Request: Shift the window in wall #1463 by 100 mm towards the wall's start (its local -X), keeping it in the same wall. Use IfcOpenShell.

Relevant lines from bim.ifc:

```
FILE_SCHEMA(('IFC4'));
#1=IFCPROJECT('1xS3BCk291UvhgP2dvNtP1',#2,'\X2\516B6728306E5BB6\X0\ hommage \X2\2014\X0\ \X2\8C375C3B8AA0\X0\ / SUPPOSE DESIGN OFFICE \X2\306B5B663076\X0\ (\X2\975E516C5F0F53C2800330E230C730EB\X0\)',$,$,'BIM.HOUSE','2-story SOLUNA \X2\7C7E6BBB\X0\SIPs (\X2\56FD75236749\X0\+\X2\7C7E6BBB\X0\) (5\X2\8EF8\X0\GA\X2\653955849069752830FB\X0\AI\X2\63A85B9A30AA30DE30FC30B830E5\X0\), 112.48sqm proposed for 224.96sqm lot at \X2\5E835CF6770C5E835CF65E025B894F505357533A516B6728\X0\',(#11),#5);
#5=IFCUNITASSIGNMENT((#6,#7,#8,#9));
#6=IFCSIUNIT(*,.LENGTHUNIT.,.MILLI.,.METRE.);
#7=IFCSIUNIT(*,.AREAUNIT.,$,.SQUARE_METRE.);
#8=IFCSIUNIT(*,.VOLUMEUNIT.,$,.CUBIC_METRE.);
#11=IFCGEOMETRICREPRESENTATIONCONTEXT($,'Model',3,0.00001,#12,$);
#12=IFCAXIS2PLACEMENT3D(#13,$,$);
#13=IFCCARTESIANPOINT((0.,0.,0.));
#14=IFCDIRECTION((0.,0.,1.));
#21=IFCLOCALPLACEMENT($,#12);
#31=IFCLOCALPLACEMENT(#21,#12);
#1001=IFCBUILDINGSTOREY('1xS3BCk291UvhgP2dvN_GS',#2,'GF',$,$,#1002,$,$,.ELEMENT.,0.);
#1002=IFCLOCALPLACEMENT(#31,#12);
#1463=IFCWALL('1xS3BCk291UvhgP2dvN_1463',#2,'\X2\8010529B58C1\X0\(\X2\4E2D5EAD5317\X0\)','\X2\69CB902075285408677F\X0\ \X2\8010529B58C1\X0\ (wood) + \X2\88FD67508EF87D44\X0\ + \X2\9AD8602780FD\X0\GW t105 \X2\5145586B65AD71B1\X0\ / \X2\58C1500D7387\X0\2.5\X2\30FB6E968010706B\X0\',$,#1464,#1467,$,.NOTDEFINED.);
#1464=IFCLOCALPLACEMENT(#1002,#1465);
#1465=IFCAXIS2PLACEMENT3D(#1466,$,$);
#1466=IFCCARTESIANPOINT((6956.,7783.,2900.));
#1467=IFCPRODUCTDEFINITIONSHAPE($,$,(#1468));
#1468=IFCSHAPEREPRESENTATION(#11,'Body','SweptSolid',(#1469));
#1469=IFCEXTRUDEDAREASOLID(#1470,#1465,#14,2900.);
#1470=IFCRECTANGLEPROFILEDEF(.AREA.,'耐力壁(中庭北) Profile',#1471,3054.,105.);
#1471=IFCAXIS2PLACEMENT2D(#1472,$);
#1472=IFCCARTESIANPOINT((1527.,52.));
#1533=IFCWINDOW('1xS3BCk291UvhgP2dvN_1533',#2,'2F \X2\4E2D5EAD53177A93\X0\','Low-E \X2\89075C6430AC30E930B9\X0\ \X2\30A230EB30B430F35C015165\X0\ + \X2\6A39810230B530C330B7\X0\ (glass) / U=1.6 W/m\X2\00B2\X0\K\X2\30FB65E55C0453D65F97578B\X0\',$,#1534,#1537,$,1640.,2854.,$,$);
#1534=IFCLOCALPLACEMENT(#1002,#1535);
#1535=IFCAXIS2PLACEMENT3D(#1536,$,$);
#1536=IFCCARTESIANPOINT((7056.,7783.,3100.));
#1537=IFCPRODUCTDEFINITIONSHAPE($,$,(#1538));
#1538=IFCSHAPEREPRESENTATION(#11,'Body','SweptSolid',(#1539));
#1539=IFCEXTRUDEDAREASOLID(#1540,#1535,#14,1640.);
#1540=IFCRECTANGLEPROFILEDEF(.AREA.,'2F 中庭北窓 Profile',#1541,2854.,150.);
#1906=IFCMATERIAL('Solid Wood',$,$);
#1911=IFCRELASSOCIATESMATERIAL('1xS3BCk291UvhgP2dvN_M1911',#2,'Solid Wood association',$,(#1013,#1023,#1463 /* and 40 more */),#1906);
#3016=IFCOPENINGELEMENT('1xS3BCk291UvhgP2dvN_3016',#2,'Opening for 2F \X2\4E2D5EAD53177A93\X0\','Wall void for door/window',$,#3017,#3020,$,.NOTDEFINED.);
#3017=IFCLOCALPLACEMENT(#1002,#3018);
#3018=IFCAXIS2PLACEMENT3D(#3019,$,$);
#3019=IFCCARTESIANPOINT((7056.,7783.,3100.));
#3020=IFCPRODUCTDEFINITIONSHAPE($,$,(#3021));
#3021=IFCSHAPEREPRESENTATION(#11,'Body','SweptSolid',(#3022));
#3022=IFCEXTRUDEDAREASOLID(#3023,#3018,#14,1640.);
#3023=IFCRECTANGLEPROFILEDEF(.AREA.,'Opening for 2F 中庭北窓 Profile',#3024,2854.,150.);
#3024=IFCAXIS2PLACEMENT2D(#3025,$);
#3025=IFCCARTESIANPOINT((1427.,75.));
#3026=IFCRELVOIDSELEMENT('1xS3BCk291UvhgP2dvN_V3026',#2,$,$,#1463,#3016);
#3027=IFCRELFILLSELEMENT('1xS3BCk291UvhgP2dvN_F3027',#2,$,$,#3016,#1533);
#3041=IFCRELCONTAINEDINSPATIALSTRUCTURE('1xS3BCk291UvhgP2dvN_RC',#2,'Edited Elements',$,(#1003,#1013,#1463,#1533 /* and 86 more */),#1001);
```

```python
import ifcopenshell
import ifcopenshell.api.geometry
import ifcopenshell.util.placement
import ifcopenshell.util.unit

model = ifcopenshell.open("bim.ifc")
unit_scale = ifcopenshell.util.unit.calculate_unit_scale(model)

window = model.by_guid("1xS3BCk291UvhgP2dvN_1533")
opening = window.FillsVoids[0].RelatingOpeningElement
wall = opening.VoidsElements[0].RelatingBuildingElement

wall_matrix = ifcopenshell.util.placement.get_local_placement(wall.ObjectPlacement)
shift = wall_matrix[:3, 0] * -0.1 / unit_scale
before = ifcopenshell.util.placement.get_local_placement(window.ObjectPlacement)[:3, 3].copy()

# The window is not placed relative to its opening, so move both.
for product in (opening, window):
    matrix = ifcopenshell.util.placement.get_local_placement(product.ObjectPlacement)
    matrix[:3, 3] += shift
    ifcopenshell.api.geometry.edit_object_placement(model, product=product, matrix=matrix, is_si=False)

after = ifcopenshell.util.placement.get_local_placement(window.ObjectPlacement)[:3, 3]
print("window moved by", (after - before).round(3) + 0.0)

model.write("bim-out.ifc")
```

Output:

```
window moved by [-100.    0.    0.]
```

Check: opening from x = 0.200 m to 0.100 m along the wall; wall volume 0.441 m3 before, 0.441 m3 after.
